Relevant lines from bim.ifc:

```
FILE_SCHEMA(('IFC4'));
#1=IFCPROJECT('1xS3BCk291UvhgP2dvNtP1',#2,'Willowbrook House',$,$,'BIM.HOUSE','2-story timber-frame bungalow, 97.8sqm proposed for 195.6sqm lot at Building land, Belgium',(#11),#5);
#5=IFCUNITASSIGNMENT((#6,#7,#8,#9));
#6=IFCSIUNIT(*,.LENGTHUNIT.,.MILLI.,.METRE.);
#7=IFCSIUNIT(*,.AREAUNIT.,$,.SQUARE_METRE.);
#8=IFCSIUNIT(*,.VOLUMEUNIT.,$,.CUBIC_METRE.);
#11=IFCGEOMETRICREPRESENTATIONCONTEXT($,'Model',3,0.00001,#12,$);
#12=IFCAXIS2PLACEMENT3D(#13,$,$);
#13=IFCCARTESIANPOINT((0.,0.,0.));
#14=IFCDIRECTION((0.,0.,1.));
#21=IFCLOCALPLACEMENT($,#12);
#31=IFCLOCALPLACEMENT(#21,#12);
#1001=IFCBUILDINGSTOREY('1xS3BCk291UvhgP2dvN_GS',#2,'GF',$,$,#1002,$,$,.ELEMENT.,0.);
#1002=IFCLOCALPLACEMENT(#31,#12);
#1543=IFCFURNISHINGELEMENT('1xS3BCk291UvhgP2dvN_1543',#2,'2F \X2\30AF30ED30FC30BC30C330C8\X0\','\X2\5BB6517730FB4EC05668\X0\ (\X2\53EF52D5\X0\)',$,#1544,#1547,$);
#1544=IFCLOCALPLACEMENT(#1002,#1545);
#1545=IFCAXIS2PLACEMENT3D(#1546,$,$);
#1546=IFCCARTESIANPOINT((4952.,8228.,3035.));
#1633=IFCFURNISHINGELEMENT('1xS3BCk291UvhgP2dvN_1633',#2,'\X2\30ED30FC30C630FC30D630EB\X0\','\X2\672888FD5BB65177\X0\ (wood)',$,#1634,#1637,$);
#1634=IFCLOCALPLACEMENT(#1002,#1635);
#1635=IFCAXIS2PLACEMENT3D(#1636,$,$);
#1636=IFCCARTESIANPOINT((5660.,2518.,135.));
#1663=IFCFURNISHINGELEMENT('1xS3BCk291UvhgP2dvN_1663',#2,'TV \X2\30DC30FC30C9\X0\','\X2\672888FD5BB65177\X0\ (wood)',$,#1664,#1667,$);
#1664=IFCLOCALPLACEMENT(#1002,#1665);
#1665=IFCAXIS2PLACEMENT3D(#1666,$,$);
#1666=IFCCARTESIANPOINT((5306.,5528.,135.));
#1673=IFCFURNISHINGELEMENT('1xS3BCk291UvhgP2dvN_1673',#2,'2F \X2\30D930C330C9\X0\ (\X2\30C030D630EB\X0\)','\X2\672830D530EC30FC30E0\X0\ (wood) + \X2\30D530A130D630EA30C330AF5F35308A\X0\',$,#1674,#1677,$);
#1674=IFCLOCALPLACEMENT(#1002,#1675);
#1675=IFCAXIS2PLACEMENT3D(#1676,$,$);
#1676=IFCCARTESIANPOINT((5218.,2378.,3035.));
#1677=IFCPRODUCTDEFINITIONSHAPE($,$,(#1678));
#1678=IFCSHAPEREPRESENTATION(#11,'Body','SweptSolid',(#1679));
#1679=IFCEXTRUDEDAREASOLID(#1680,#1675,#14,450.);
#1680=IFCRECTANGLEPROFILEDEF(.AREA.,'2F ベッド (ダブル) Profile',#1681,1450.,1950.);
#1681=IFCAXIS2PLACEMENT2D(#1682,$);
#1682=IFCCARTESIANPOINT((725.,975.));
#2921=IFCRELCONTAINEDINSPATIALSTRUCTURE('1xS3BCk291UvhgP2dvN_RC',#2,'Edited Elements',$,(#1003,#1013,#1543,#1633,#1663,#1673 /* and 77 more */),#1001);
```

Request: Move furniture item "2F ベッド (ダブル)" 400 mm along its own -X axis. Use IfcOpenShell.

```python
import ifcopenshell
import ifcopenshell.api.geometry
import ifcopenshell.util.placement
import ifcopenshell.util.unit

model = ifcopenshell.open("bim.ifc")
unit_scale = ifcopenshell.util.unit.calculate_unit_scale(model)

item = model.by_id(1673)
matrix = ifcopenshell.util.placement.get_local_placement(item.ObjectPlacement)
matrix[:3, 3] -= matrix[:3, 0] * 0.4 / unit_scale
ifcopenshell.api.geometry.edit_object_placement(model, product=item, matrix=matrix, is_si=False)

print(ifcopenshell.util.placement.get_local_placement(item.ObjectPlacement).round(3) + 0.0)

model.write("bim_v2.ifc")
```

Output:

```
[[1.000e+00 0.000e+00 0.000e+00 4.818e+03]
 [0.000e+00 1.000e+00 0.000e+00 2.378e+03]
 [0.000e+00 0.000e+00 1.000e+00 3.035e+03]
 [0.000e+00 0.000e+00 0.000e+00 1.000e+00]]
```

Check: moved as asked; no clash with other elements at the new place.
